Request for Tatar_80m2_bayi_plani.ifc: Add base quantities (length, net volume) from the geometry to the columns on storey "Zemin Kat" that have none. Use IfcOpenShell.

First a look at what the model holds.

```python
import ifcopenshell
import ifcopenshell.util.element
import ifcopenshell.util.unit

model = ifcopenshell.open("Tatar_80m2_bayi_plani.ifc")
print(model.schema)
for unit_type in ("LENGTHUNIT", "AREAUNIT", "VOLUMEUNIT"):
    print(unit_type, ifcopenshell.util.unit.calculate_unit_scale(model, unit_type))
storey = next(s for s in model.by_type("IfcBuildingStorey") if s.Name == "Zemin Kat")
columns = [e for e in ifcopenshell.util.element.get_decomposition(storey) if e.is_a("IfcColumn")]
for e in sorted(columns, key=lambda e: e.id()):
    print(e.id(), e.is_a(), e.Name, list(ifcopenshell.util.element.get_psets(e, qtos_only=True)), sep=" | ")
```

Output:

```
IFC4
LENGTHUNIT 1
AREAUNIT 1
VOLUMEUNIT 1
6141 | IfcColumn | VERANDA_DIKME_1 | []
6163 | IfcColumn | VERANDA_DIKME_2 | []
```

```python
import ifcopenshell
import ifcopenshell.api.pset
import ifcopenshell.geom
import ifcopenshell.util.element
import ifcopenshell.util.shape
import ifcopenshell.util.unit

model = ifcopenshell.open("Tatar_80m2_bayi_plani.ifc")
unit_scale = ifcopenshell.util.unit.calculate_unit_scale(model)
volume_scale = ifcopenshell.util.unit.calculate_unit_scale(model, "VOLUMEUNIT")
settings = ifcopenshell.geom.settings()

storey = next(s for s in model.by_type("IfcBuildingStorey") if s.Name == "Zemin Kat")
columns = [e for e in ifcopenshell.util.element.get_decomposition(storey) if e.is_a("IfcColumn")]

for e in sorted(columns, key=lambda e: e.id()):
    if ifcopenshell.util.element.get_psets(e, qtos_only=True, should_inherit=False):
        continue
    # Geometry comes back in metres, in the element's own axes.
    shape = ifcopenshell.geom.create_shape(settings, e)
    values = {
        "Length": ifcopenshell.util.shape.get_z(shape.geometry) / unit_scale,
        "NetVolume": ifcopenshell.util.shape.get_volume(shape.geometry) / volume_scale,
    }
    qto = ifcopenshell.api.pset.add_qto(model, product=e, name="Qto_ColumnBaseQuantities")
    ifcopenshell.api.pset.edit_qto(model, qto=qto, properties=values)
    print(e.id(), {k: round(v, 3) for k, v in values.items()})

model.write("Tatar_80m2_bayi_plani_rev.ifc")
```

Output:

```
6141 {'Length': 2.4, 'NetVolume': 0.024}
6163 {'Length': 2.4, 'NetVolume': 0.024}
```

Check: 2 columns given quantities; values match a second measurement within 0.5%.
